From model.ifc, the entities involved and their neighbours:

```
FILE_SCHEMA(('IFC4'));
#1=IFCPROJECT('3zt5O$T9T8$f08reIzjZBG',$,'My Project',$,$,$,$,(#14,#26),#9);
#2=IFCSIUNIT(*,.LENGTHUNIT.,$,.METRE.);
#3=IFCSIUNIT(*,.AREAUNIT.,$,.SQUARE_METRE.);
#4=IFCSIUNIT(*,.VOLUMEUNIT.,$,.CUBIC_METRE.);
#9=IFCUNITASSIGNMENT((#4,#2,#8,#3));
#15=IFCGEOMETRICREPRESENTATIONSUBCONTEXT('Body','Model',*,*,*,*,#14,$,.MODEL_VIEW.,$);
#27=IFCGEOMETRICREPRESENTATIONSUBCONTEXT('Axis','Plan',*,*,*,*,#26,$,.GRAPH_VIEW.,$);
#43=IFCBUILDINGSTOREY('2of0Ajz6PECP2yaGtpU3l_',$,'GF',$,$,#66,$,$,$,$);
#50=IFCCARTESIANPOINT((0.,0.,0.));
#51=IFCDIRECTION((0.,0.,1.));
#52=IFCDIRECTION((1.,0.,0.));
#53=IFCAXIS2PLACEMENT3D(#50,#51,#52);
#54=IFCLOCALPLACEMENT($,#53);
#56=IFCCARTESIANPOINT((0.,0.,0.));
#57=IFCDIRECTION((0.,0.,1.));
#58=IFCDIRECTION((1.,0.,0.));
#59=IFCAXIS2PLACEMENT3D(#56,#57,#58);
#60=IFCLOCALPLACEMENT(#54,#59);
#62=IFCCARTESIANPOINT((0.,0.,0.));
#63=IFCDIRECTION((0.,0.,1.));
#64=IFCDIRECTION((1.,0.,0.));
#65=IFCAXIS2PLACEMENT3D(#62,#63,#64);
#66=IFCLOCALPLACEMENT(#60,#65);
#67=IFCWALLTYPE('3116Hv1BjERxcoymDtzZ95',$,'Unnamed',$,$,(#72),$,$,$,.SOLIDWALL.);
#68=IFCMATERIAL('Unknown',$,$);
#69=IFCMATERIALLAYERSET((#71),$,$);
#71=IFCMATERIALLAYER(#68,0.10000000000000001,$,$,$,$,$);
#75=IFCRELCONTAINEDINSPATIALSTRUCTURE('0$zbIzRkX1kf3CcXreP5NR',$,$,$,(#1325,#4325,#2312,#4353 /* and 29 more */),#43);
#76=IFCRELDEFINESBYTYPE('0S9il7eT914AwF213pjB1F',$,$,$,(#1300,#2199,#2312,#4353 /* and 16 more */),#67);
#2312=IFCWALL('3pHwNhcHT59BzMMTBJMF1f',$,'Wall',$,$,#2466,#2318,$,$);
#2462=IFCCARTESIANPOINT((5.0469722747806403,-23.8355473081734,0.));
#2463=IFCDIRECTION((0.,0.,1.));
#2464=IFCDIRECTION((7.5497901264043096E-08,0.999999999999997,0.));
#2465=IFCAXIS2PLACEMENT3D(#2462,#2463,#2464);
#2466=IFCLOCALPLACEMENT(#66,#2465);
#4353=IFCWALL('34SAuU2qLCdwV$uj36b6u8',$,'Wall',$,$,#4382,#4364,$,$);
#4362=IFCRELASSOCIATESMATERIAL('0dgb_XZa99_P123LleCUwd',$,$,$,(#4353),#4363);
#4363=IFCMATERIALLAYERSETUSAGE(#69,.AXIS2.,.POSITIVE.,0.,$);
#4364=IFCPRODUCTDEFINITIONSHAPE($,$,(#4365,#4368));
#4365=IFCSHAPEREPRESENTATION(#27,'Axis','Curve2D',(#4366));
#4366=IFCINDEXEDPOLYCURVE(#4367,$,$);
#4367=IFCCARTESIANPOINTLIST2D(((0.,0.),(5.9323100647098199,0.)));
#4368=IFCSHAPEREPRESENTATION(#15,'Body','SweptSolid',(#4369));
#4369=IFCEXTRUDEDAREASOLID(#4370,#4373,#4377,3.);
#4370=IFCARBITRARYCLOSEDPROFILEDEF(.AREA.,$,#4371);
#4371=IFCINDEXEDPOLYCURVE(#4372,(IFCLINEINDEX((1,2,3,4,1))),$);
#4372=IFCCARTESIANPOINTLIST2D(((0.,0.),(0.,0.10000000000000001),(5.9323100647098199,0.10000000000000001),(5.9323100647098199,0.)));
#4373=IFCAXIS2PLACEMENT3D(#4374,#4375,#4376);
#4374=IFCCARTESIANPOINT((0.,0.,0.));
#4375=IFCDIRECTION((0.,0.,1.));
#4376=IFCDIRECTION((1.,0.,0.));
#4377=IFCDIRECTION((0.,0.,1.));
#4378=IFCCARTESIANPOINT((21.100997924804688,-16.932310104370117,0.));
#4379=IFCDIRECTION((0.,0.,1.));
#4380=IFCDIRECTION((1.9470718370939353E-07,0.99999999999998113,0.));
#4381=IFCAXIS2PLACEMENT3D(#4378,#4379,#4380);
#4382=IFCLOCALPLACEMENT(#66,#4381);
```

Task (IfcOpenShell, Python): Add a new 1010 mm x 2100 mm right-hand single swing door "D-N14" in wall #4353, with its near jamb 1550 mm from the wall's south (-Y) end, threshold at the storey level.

```python
import numpy as np
import ifcopenshell
import ifcopenshell.api.feature
import ifcopenshell.api.geometry
import ifcopenshell.api.root
import ifcopenshell.api.spatial
import ifcopenshell.geom
import ifcopenshell.util.element
import ifcopenshell.util.placement
import ifcopenshell.util.representation
import ifcopenshell.util.shape
import ifcopenshell.util.unit

model = ifcopenshell.open("model.ifc")
unit_scale = ifcopenshell.util.unit.calculate_unit_scale(model)
settings = ifcopenshell.geom.settings()


def volume(element):
    """Net volume in cubic metres, openings subtracted."""
    shape = ifcopenshell.geom.create_shape(settings, element)
    return ifcopenshell.util.shape.get_volume(shape.geometry)


wall = model.by_guid("34SAuU2qLCdwV$uj36b6u8")
storey = ifcopenshell.util.element.get_container(wall, ifc_class="IfcBuildingStorey")
context = ifcopenshell.util.representation.get_context(model, "Model", "Body", "MODEL_VIEW")
before = volume(wall)

width, height, from_end, sill = 1.01, 2.1, 1.55, 0.0  # metres

# The wall runs along its own X axis, and the end named is its -X end.
wall_shape = ifcopenshell.geom.create_shape(settings, wall)
x, y, z = ifcopenshell.util.shape.get_vertices(wall_shape.geometry).T
start = x.min() + from_end
face, thickness = float(y.min()), float(y.max() - y.min())
wall_matrix = ifcopenshell.util.placement.get_local_placement(wall.ObjectPlacement)
level = ifcopenshell.util.placement.get_local_placement(storey.ObjectPlacement)[2, 3]


def in_wall(x, y):
    """Placement at x, y metres in the wall's axes, at sill height."""
    matrix = wall_matrix.copy()
    matrix[:, 3] = wall_matrix @ np.array([x / unit_scale, y / unit_scale, 0.0, 1.0])
    matrix[2, 3] = level + sill / unit_scale
    return matrix


# Opening: a box that overshoots both wall faces by 50 mm.
opening = ifcopenshell.api.root.create_entity(model, ifc_class="IfcOpeningElement", predefined_type="OPENING")
box = ifcopenshell.api.geometry.add_wall_representation(
    model, context=context, length=width, height=height, thickness=thickness + 0.1
)
ifcopenshell.api.geometry.assign_representation(model, product=opening, representation=box)
ifcopenshell.api.geometry.edit_object_placement(model, product=opening, matrix=in_wall(start, face - 0.05), is_si=False)
ifcopenshell.api.feature.add_feature(model, feature=opening, element=wall)

door = ifcopenshell.api.root.create_entity(model, ifc_class="IfcDoor", name="D-N14", predefined_type="DOOR")
door.OverallWidth, door.OverallHeight = width / unit_scale, height / unit_scale
door.OperationType = "SINGLE_SWING_RIGHT"
body = ifcopenshell.api.geometry.add_door_representation(
    model,
    context=context,
    overall_width=door.OverallWidth,
    overall_height=door.OverallHeight,
    operation_type="SINGLE_SWING_RIGHT",
    lining_properties={"LiningDepth": thickness / unit_scale, "ThresholdDepth": thickness / unit_scale},
)
ifcopenshell.api.geometry.assign_representation(model, product=door, representation=body)
ifcopenshell.api.spatial.assign_container(model, products=[door], relating_structure=storey)
ifcopenshell.api.feature.add_filling(model, opening=opening, element=door)

# The lining spans the wall, so the door starts at the wall face.
ifcopenshell.api.geometry.edit_object_placement(model, product=door, matrix=in_wall(start, face), is_si=False)

after = volume(wall)

print(f"wall volume {before:.3f} -> {after:.3f} m3")

model.write("model_edited.ifc")
```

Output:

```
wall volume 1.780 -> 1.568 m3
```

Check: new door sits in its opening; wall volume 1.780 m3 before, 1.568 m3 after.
